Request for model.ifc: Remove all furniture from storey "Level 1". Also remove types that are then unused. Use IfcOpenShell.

First a look at what the model holds.

```python
import ifcopenshell
import ifcopenshell.util.element

model = ifcopenshell.open("model.ifc")
print(model.schema)
storey = next(s for s in model.by_type("IfcBuildingStorey") if s.Name == "Level 1")
furniture = [e for e in ifcopenshell.util.element.get_decomposition(storey) if e.is_a("IfcFurnishingElement")]
seen = {}
for e in furniture:
    element_type = ifcopenshell.util.element.get_type(e)
    name = element_type.Name if element_type not in (None, e) else None
    seen[name] = seen.get(name, 0) + 1
for name, count in sorted(seen.items(), key=str):
    print(count, "x", name)
```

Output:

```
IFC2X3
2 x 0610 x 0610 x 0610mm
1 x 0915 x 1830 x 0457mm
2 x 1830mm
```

```python
import ifcopenshell
import ifcopenshell.api.root
import ifcopenshell.util.element

model = ifcopenshell.open("model.ifc")

storey = next(s for s in model.by_type("IfcBuildingStorey") if s.Name == "Level 1")
furniture = [e for e in ifcopenshell.util.element.get_decomposition(storey) if e.is_a("IfcFurnishingElement")]
types = {ifcopenshell.util.element.get_type(e) for e in furniture} - {None, *furniture}

for e in furniture:
    ifcopenshell.api.root.remove_product(model, product=e)
print(len(furniture), "removed")

unused = [t for t in types if not ifcopenshell.util.element.get_types(t)]
for t in unused:
    ifcopenshell.api.root.remove_product(model, product=t)
print(len(unused), "unused types removed")

model.write("model_updated.ifc")
```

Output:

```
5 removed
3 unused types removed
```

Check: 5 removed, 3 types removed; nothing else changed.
